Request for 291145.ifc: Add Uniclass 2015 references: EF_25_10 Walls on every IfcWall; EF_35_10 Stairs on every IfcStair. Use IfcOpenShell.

First a look at what the model holds.

```python
import ifcopenshell

model = ifcopenshell.open("291145.ifc")
print(model.schema)
print("classifications:", [c.Name for c in model.by_type("IfcClassification")])
for ifc_class in ("IfcDoor", "IfcRoof", "IfcStair", "IfcWall", "IfcWindow"):
    print(ifc_class, len(model.by_type(ifc_class)))
```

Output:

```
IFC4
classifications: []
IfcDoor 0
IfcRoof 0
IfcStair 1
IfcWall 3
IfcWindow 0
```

```python
import ifcopenshell
import ifcopenshell.api.classification

model = ifcopenshell.open("291145.ifc")

system = ifcopenshell.api.classification.add_classification(model, classification="Uniclass 2015")

codes = {
    "IfcWall": ("EF_25_10", "Walls"),
    "IfcStair": ("EF_35_10", "Stairs"),
}
for ifc_class, (code, name) in codes.items():
    products = model.by_type(ifc_class)
    ifcopenshell.api.classification.add_reference(
        model, products=products, classification=system, identification=code, name=name
    )
    print(code, len(products))

model.write("291145-out.ifc")
```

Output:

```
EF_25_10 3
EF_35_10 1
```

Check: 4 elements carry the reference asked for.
